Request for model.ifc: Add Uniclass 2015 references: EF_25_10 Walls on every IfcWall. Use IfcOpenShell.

First a look at what the model holds.

```python
import ifcopenshell

model = ifcopenshell.open("model.ifc")
print(model.schema)
print("classifications:", [c.Name for c in model.by_type("IfcClassification")])
for ifc_class in ("IfcDoor", "IfcRoof", "IfcStair", "IfcWall", "IfcWindow"):
    print(ifc_class, len(model.by_type(ifc_class)))
```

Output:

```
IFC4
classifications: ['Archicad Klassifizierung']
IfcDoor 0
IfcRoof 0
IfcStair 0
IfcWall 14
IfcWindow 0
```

```python
import ifcopenshell
import ifcopenshell.api.classification

model = ifcopenshell.open("model.ifc")

system = ifcopenshell.api.classification.add_classification(model, classification="Uniclass 2015")

codes = {
    "IfcWall": ("EF_25_10", "Walls"),
}
for ifc_class, (code, name) in codes.items():
    products = model.by_type(ifc_class)
    ifcopenshell.api.classification.add_reference(
        model, products=products, classification=system, identification=code, name=name
    )
    print(code, len(products))

model.write("model_v2.ifc")
```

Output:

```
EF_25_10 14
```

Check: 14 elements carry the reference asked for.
